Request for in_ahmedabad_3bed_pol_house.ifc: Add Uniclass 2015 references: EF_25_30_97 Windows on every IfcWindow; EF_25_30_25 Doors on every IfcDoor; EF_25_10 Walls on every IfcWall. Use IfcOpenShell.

First a look at what the model holds.

```python
import ifcopenshell

model = ifcopenshell.open("in_ahmedabad_3bed_pol_house.ifc")
print(model.schema)
print("classifications:", [c.Name for c in model.by_type("IfcClassification")])
for ifc_class in ("IfcDoor", "IfcRoof", "IfcStair", "IfcWall", "IfcWindow"):
    print(ifc_class, len(model.by_type(ifc_class)))
```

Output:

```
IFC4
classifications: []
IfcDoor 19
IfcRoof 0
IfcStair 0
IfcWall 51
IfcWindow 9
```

```python
import ifcopenshell
import ifcopenshell.api.classification

model = ifcopenshell.open("in_ahmedabad_3bed_pol_house.ifc")

system = ifcopenshell.api.classification.add_classification(model, classification="Uniclass 2015")

codes = {
    "IfcWindow": ("EF_25_30_97", "Windows"),
    "IfcDoor": ("EF_25_30_25", "Doors"),
    "IfcWall": ("EF_25_10", "Walls"),
}
for ifc_class, (code, name) in codes.items():
    products = model.by_type(ifc_class)
    ifcopenshell.api.classification.add_reference(
        model, products=products, classification=system, identification=code, name=name
    )
    print(code, len(products))

model.write("in_ahmedabad_3bed_pol_house_updated.ifc")
```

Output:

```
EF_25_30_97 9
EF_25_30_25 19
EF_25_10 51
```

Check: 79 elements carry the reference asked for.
